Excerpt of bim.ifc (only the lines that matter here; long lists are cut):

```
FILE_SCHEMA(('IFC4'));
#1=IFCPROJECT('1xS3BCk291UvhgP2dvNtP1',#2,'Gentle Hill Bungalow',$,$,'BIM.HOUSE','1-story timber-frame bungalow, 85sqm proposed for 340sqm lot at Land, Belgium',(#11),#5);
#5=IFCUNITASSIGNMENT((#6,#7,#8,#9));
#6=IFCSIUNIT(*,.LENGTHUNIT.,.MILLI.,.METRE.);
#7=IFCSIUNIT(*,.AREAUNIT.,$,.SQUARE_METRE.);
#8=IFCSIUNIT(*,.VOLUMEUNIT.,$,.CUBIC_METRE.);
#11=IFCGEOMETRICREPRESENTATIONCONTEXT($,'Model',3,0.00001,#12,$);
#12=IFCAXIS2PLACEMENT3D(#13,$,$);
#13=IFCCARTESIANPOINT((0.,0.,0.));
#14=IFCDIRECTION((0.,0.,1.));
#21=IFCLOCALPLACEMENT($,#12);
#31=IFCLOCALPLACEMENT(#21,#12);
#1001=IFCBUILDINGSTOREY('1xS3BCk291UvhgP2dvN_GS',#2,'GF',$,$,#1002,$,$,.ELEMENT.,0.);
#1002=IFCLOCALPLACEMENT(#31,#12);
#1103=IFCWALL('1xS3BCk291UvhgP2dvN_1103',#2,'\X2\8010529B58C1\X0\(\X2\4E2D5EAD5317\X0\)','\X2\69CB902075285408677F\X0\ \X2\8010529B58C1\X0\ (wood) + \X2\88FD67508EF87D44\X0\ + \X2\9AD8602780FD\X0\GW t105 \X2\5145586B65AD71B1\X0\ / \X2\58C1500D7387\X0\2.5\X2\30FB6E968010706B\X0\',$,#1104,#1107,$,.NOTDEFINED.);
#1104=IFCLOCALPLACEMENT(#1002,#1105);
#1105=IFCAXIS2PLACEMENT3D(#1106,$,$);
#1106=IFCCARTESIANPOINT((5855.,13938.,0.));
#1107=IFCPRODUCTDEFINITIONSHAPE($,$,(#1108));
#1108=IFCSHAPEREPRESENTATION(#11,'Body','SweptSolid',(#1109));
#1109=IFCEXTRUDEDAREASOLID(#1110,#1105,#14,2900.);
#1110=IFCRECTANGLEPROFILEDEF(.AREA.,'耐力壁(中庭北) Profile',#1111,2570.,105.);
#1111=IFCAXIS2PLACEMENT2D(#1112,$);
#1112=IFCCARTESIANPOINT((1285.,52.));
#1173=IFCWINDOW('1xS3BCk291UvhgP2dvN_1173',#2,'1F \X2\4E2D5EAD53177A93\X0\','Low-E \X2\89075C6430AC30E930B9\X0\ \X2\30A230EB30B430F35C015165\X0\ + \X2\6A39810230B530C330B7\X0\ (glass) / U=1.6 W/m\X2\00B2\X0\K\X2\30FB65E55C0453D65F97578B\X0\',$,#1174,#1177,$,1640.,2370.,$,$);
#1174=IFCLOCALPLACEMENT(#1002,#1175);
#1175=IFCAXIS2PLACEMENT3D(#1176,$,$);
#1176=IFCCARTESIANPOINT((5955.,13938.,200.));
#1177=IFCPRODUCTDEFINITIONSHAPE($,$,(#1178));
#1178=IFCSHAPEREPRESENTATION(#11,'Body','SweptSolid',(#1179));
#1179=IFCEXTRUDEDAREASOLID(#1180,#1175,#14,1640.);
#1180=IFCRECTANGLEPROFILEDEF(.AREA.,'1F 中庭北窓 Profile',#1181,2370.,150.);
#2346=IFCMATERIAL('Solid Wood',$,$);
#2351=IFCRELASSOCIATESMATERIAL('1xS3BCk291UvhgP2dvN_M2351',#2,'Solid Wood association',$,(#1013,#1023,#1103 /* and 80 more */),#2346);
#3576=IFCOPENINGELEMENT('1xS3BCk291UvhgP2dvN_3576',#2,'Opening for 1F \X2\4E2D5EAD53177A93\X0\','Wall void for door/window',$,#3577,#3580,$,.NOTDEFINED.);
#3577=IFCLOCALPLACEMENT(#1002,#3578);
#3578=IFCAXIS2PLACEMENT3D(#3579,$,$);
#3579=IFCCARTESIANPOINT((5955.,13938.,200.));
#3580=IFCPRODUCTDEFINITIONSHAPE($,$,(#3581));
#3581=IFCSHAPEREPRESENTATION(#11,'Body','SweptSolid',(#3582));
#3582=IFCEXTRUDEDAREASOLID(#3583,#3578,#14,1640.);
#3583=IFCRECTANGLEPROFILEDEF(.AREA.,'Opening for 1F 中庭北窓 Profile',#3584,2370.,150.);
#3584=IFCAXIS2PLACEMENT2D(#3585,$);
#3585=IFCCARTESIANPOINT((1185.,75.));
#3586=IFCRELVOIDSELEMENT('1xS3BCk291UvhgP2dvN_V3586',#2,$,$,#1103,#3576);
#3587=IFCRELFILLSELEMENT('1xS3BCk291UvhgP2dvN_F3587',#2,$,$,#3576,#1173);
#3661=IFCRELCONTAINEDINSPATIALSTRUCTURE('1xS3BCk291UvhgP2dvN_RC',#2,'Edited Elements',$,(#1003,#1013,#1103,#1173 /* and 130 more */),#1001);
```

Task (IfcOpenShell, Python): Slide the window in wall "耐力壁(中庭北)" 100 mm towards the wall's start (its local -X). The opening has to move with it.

```python
import ifcopenshell
import ifcopenshell.api.geometry
import ifcopenshell.util.placement
import ifcopenshell.util.unit

model = ifcopenshell.open("bim.ifc")
unit_scale = ifcopenshell.util.unit.calculate_unit_scale(model)

window = model.by_guid("1xS3BCk291UvhgP2dvN_1173")
opening = window.FillsVoids[0].RelatingOpeningElement
wall = opening.VoidsElements[0].RelatingBuildingElement

wall_matrix = ifcopenshell.util.placement.get_local_placement(wall.ObjectPlacement)
shift = wall_matrix[:3, 0] * -0.1 / unit_scale
before = ifcopenshell.util.placement.get_local_placement(window.ObjectPlacement)[:3, 3].copy()

# The window is not placed relative to its opening, so move both.
for product in (opening, window):
    matrix = ifcopenshell.util.placement.get_local_placement(product.ObjectPlacement)
    matrix[:3, 3] += shift
    ifcopenshell.api.geometry.edit_object_placement(model, product=product, matrix=matrix, is_si=False)

after = ifcopenshell.util.placement.get_local_placement(window.ObjectPlacement)[:3, 3]
print("window moved by", (after - before).round(3) + 0.0)

model.write("bim-out.ifc")
```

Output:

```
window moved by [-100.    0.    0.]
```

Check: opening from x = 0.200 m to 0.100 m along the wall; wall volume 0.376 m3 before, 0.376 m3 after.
